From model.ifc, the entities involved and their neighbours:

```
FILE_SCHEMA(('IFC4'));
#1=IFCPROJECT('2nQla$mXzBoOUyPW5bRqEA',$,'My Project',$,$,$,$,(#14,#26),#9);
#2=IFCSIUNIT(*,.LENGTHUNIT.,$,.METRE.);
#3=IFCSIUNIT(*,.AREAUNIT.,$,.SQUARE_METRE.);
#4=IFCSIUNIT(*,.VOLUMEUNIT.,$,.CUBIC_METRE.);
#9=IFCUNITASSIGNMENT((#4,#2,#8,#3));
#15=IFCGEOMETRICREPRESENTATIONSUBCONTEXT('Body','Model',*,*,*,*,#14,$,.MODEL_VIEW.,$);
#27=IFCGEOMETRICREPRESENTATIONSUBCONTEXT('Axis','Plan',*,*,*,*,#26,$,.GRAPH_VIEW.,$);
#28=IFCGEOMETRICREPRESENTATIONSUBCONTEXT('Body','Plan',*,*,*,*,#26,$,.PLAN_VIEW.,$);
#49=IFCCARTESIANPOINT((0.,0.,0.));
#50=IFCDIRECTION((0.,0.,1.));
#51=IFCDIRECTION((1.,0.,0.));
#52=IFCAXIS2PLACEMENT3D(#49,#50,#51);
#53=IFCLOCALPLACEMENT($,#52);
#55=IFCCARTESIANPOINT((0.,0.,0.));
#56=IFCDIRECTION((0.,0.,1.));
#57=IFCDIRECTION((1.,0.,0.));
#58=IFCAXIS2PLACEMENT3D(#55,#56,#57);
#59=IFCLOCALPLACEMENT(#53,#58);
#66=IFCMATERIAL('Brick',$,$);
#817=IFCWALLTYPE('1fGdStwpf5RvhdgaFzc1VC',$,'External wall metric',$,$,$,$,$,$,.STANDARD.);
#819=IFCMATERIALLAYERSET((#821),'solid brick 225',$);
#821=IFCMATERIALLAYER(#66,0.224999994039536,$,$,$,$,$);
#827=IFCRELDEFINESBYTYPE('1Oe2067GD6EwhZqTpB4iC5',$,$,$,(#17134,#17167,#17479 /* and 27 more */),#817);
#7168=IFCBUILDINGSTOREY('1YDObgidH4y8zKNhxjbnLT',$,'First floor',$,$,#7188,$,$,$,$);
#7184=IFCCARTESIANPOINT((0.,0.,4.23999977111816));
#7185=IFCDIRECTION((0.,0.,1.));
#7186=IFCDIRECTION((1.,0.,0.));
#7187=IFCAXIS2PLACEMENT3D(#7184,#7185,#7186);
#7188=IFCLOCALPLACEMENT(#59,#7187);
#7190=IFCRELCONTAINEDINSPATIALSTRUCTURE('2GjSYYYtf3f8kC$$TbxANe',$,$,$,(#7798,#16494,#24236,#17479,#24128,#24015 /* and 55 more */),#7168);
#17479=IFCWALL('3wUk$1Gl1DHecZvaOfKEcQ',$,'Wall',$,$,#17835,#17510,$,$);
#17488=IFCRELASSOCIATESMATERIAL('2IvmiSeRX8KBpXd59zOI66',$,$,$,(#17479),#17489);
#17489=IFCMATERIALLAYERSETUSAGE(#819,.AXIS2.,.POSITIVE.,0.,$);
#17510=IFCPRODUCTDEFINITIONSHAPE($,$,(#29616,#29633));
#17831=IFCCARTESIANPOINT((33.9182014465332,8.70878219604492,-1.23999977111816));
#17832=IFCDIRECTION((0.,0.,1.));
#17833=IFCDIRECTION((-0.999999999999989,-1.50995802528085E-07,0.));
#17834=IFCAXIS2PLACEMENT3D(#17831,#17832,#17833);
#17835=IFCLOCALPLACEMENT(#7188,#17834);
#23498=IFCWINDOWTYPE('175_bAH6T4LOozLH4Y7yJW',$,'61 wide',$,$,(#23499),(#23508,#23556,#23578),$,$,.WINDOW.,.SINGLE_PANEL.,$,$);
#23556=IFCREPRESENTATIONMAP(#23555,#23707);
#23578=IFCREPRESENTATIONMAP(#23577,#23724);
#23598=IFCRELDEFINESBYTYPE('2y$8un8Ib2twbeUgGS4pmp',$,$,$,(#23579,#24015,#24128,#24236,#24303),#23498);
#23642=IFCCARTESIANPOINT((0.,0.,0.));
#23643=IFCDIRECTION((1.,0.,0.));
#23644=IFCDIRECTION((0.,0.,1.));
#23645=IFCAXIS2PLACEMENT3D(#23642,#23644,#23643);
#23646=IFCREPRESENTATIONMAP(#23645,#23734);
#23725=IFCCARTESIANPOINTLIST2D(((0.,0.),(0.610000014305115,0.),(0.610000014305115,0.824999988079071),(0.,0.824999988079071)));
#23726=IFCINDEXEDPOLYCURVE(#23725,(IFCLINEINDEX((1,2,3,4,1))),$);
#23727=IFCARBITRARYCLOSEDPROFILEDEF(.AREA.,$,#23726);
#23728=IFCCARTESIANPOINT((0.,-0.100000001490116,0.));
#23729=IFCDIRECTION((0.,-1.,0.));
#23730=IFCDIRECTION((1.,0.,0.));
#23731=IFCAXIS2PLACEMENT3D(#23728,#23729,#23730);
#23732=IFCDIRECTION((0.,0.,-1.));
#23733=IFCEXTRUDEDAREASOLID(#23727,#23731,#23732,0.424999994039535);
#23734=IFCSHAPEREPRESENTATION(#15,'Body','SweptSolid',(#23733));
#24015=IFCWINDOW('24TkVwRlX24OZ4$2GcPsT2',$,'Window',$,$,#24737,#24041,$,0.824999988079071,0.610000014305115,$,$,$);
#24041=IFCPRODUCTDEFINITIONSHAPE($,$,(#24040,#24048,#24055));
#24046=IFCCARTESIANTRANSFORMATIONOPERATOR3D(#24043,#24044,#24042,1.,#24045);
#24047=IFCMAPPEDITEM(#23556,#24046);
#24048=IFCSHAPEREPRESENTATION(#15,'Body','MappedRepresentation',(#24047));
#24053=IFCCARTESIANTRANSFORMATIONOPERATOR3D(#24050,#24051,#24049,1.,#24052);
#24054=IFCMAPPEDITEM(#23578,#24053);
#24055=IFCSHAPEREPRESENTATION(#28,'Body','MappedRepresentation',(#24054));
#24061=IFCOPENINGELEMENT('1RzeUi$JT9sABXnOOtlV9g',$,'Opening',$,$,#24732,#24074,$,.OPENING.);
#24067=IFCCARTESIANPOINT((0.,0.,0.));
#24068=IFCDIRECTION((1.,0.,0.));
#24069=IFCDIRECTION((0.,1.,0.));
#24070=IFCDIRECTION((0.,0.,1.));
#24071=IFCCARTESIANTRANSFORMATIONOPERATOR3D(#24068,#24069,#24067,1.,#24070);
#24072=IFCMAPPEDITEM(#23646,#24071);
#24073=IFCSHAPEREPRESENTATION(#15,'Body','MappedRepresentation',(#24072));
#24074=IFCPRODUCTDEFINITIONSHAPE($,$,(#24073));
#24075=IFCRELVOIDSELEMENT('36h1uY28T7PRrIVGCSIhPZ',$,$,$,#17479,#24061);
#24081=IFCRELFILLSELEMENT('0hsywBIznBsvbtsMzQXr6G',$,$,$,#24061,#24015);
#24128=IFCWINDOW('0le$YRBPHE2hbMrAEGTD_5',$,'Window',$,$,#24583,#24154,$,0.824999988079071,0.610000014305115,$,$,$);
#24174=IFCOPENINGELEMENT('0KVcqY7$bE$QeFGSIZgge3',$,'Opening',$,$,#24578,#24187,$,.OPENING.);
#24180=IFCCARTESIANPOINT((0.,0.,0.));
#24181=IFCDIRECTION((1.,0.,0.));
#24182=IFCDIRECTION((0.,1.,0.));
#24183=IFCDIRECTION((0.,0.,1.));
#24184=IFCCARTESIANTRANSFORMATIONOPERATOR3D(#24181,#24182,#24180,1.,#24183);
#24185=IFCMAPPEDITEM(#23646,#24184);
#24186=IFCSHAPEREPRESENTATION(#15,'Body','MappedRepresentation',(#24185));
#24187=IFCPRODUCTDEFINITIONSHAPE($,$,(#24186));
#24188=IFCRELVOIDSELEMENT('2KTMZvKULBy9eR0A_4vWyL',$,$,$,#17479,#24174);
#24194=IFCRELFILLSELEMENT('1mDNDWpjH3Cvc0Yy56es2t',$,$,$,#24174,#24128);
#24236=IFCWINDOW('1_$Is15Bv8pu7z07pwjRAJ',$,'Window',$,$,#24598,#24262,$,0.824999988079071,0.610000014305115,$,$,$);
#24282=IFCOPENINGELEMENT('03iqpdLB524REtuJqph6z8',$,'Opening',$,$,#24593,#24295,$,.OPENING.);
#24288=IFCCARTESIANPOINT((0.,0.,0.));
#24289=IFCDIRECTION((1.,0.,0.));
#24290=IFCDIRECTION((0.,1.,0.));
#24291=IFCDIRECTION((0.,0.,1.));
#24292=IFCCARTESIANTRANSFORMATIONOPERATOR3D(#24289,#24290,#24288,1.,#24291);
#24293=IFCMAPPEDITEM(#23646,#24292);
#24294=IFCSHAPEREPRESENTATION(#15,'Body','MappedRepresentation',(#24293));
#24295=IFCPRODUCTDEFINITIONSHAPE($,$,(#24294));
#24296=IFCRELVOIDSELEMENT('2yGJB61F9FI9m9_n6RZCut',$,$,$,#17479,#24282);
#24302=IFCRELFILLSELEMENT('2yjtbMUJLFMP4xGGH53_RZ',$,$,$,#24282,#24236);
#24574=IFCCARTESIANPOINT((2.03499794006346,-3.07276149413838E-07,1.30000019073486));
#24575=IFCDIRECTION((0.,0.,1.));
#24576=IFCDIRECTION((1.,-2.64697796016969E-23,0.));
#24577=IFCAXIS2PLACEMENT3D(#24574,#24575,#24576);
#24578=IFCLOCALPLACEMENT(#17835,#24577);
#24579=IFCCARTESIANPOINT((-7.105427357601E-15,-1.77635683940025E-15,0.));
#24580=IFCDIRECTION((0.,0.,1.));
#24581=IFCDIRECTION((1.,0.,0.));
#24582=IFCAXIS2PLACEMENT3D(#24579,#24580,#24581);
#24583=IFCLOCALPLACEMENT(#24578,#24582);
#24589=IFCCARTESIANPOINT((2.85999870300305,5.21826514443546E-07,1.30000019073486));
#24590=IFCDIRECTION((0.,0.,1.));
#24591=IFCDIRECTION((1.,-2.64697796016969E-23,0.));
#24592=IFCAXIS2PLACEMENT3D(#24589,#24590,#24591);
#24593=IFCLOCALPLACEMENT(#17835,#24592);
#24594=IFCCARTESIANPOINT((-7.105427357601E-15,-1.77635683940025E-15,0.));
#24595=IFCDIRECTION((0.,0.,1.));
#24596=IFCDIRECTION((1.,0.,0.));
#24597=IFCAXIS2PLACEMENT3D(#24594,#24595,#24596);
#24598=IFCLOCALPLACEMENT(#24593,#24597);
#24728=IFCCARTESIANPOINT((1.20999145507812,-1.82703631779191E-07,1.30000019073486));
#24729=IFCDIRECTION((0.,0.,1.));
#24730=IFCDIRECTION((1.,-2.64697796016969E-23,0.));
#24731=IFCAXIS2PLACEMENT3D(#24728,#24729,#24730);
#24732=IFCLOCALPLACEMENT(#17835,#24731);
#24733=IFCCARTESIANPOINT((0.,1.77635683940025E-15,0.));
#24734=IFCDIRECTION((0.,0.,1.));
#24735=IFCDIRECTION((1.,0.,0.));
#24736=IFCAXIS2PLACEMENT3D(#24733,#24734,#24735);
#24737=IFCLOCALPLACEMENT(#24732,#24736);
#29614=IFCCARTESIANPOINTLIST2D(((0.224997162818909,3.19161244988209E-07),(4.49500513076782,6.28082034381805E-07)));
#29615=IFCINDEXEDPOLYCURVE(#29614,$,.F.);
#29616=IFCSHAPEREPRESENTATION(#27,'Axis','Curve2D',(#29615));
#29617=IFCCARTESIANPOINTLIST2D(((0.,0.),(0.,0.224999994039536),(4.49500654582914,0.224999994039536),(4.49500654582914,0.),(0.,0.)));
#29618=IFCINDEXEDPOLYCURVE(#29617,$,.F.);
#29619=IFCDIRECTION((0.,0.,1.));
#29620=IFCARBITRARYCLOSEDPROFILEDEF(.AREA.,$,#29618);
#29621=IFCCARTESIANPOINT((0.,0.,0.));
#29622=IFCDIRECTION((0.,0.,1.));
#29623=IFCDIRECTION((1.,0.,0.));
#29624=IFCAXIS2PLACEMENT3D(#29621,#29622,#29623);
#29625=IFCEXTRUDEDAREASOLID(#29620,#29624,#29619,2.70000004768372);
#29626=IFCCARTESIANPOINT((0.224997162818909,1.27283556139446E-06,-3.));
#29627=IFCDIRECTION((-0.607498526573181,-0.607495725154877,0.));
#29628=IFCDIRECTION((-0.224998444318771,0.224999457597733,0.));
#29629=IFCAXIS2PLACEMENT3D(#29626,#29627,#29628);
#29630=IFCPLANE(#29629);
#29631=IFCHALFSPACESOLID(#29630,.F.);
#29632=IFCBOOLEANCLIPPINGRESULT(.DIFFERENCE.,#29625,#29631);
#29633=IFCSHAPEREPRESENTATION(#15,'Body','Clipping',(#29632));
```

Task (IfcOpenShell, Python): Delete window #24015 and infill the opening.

```python
import ifcopenshell
import ifcopenshell.api.feature
import ifcopenshell.api.root
import ifcopenshell.geom
import ifcopenshell.util.shape

model = ifcopenshell.open("model.ifc")
settings = ifcopenshell.geom.settings()


def volume(element):
    """Net volume in cubic metres, openings subtracted."""
    shape = ifcopenshell.geom.create_shape(settings, element)
    return ifcopenshell.util.shape.get_volume(shape.geometry)


window = model.by_guid("24TkVwRlX24OZ4$2GcPsT2")
opening = window.FillsVoids[0].RelatingOpeningElement
wall = opening.VoidsElements[0].RelatingBuildingElement
before = volume(wall)

ifcopenshell.api.root.remove_product(model, product=window)
ifcopenshell.api.feature.remove_feature(model, feature=opening)

after = volume(wall)

print(f"wall volume {before:.3f} -> {after:.3f} m3")

model.write("model_rev.ifc")
```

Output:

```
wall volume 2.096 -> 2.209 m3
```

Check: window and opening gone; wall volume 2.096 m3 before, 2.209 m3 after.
